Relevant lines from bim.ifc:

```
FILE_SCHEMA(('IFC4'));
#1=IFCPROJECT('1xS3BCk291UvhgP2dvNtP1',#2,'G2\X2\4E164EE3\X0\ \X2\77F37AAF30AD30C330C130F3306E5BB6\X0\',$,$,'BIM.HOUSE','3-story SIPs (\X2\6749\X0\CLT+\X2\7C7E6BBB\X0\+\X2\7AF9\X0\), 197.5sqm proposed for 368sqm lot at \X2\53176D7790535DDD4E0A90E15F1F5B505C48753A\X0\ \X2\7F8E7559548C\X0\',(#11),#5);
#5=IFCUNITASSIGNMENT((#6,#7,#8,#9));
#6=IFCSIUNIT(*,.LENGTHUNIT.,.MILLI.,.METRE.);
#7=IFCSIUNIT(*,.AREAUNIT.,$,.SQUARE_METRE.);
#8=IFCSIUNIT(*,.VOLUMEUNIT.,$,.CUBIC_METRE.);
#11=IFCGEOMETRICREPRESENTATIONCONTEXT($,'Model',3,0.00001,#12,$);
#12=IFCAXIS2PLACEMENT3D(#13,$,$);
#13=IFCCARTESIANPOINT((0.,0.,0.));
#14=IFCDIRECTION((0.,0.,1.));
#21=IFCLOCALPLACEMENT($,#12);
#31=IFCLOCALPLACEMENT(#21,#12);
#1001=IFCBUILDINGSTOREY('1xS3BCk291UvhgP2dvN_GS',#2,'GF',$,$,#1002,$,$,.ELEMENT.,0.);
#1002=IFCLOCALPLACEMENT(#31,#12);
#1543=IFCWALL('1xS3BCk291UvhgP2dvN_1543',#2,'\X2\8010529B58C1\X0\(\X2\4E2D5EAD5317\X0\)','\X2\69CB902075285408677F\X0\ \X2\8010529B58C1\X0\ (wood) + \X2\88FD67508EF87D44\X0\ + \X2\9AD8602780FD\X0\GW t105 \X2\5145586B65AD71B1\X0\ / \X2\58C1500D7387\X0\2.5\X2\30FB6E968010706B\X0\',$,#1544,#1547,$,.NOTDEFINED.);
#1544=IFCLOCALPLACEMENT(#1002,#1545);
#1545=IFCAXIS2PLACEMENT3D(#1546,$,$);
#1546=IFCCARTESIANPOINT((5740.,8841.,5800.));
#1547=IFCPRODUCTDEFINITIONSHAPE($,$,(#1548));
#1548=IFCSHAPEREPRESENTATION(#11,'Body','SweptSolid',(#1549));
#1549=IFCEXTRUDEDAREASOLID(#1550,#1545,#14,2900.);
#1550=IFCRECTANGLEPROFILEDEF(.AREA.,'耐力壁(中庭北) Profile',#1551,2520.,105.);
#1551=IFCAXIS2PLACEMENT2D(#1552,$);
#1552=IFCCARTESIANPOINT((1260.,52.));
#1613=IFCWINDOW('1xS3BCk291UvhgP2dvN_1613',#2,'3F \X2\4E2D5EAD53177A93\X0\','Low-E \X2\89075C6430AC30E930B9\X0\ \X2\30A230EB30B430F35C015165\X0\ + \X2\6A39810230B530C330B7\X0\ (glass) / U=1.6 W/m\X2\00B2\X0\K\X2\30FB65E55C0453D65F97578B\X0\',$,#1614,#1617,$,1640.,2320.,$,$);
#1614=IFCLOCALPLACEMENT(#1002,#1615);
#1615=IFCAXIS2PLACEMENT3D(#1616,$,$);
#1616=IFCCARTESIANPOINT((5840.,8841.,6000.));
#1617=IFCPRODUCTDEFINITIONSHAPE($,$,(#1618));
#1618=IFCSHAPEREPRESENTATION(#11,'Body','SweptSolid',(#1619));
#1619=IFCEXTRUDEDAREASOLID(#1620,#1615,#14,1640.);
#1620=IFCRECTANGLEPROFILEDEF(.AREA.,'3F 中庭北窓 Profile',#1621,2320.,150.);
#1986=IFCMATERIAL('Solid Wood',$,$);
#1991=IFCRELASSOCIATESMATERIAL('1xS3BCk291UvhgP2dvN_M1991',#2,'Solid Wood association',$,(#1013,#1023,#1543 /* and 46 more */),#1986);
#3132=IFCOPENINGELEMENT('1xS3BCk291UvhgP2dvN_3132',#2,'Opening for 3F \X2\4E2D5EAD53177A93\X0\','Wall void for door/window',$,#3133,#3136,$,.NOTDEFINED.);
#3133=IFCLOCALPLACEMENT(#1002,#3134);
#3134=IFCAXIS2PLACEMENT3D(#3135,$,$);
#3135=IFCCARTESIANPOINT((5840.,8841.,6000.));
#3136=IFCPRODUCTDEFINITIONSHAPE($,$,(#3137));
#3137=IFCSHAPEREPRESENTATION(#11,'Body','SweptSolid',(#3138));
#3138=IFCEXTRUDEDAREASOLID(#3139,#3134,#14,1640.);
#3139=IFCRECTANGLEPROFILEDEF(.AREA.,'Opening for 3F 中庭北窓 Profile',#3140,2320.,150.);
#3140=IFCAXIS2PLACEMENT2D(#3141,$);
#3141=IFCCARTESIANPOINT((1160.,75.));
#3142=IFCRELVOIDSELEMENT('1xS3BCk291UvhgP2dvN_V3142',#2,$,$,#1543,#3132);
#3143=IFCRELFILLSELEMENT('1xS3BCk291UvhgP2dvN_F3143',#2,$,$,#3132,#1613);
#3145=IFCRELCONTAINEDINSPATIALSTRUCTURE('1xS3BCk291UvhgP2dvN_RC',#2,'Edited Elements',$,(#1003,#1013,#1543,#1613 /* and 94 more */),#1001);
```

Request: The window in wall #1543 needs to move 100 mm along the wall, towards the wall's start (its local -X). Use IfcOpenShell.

```python
import ifcopenshell
import ifcopenshell.api.geometry
import ifcopenshell.util.placement
import ifcopenshell.util.unit

model = ifcopenshell.open("bim.ifc")
unit_scale = ifcopenshell.util.unit.calculate_unit_scale(model)

window = model.by_id(1613)
opening = window.FillsVoids[0].RelatingOpeningElement
wall = opening.VoidsElements[0].RelatingBuildingElement

wall_matrix = ifcopenshell.util.placement.get_local_placement(wall.ObjectPlacement)
shift = wall_matrix[:3, 0] * -0.1 / unit_scale
before = ifcopenshell.util.placement.get_local_placement(window.ObjectPlacement)[:3, 3].copy()

# The window is not placed relative to its opening, so move both.
for product in (opening, window):
    matrix = ifcopenshell.util.placement.get_local_placement(product.ObjectPlacement)
    matrix[:3, 3] += shift
    ifcopenshell.api.geometry.edit_object_placement(model, product=product, matrix=matrix, is_si=False)

after = ifcopenshell.util.placement.get_local_placement(window.ObjectPlacement)[:3, 3]
print("window moved by", (after - before).round(3) + 0.0)

model.write("bim_updated.ifc")
```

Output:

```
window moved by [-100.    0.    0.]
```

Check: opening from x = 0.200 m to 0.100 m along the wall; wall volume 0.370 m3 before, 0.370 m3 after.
